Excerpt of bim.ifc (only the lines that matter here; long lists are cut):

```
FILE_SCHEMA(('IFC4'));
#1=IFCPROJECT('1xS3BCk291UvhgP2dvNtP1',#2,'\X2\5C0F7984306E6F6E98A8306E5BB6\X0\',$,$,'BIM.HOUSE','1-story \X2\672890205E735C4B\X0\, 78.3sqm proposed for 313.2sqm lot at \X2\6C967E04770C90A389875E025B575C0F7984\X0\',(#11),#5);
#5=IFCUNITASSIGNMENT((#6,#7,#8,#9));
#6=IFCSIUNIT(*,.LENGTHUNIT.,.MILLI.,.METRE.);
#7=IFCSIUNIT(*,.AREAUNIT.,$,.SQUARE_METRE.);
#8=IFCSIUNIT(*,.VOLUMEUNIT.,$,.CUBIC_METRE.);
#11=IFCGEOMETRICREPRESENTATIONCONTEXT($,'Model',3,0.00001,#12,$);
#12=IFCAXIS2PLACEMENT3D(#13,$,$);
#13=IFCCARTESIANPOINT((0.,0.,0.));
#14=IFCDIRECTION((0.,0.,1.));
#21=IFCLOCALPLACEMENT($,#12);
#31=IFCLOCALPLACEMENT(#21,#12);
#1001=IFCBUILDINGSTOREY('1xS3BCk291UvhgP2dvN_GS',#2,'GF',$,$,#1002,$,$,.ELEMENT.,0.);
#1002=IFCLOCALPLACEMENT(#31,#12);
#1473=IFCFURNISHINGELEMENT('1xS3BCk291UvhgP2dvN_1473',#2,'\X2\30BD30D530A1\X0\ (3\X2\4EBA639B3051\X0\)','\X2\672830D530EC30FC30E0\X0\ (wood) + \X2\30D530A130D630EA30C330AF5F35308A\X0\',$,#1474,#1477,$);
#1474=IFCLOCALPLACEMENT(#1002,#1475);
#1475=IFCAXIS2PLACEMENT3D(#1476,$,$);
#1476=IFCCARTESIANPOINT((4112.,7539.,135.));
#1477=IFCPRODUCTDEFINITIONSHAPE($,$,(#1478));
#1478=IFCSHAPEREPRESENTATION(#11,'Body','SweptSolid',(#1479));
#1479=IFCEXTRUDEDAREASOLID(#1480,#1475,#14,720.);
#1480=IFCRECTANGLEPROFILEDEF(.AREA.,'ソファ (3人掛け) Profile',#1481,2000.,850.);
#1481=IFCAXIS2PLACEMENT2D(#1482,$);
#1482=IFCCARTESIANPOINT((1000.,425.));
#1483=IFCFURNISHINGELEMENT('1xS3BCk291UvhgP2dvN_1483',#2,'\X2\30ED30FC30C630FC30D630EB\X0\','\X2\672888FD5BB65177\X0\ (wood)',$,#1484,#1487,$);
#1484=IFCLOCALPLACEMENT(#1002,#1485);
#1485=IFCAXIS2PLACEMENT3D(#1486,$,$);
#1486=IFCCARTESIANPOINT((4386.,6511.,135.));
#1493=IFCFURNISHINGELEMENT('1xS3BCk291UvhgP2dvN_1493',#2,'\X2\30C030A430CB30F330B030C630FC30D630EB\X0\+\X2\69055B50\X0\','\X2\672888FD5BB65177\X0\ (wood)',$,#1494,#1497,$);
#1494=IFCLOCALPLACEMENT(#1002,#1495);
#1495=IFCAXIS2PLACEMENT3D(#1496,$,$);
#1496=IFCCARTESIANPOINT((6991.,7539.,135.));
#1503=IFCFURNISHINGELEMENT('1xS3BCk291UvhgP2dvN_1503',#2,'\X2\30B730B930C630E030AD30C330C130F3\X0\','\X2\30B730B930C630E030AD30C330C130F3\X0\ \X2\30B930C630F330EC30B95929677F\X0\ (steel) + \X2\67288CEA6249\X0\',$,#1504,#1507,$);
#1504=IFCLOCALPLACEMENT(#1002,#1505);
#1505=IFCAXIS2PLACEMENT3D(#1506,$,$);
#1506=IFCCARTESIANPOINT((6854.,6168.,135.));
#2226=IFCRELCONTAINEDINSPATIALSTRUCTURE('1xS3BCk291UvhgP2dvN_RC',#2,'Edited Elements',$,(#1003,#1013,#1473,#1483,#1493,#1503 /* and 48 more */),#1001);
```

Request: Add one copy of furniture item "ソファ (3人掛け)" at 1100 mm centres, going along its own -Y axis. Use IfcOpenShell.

```python
import ifcopenshell
import ifcopenshell.api.geometry
import ifcopenshell.api.root
import ifcopenshell.util.element
import ifcopenshell.util.placement
import ifcopenshell.util.unit

model = ifcopenshell.open("bim.ifc")
unit_scale = ifcopenshell.util.unit.calculate_unit_scale(model)


def reuse_history(source, copy):
    """copy_class also copies each property set's owner history, people and application; keep the originals."""
    for rel in copy.IsDefinedBy:
        if rel.is_a("IfcRelDefinesByProperties") and (history := rel.RelatingPropertyDefinition.OwnerHistory):
            rel.RelatingPropertyDefinition.OwnerHistory = source.OwnerHistory
            ifcopenshell.util.element.remove_deep2(model, history)


source = model.by_id(1473)
base = ifcopenshell.util.placement.get_local_placement(source.ObjectPlacement)
step = -base[:3, 1] * 1.1 / unit_scale

for i in range(1, 2):
    copy = ifcopenshell.api.root.copy_class(model, product=source)
    copy.Representation = ifcopenshell.util.element.copy_deep(
        model, source.Representation, exclude=["IfcGeometricRepresentationContext", "IfcRepresentationMap"]
    )
    reuse_history(source, copy)
    matrix = base.copy()
    matrix[:3, 3] += i * step
    print("added at", matrix[:3, 3].round(3) + 0.0)
    ifcopenshell.api.geometry.edit_object_placement(model, product=copy, matrix=matrix, is_si=False)

model.write("bim_rev.ifc")
```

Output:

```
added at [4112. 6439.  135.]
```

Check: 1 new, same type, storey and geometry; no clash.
